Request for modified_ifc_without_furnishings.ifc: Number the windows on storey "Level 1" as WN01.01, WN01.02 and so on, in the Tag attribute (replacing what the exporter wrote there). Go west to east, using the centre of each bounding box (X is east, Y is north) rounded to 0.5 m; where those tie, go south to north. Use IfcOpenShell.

First a look at what the model holds.

```python
import ifcopenshell
import ifcopenshell.util.element
import ifcopenshell.util.placement

model = ifcopenshell.open("modified_ifc_without_furnishings.ifc")
print(model.schema)
storey = next(s for s in model.by_type("IfcBuildingStorey") if s.Name == "Level 1")
windows = [e for e in ifcopenshell.util.element.get_decomposition(storey) if e.is_a("IfcWindow")]
for e in sorted(windows, key=lambda e: e.id()):
    origin = ifcopenshell.util.placement.get_local_placement(e.ObjectPlacement)[:3, 3]
    print(e.id(), e.Tag, e.Name, origin.round(2) + 0.0, sep=" | ")
```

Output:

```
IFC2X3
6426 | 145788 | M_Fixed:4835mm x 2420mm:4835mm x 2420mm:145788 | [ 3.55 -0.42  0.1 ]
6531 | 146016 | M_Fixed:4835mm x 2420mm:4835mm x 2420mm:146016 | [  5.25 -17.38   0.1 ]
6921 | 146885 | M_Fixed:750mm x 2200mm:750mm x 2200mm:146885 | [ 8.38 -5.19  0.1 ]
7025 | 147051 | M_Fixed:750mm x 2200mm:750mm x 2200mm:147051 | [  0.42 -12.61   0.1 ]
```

```python
import ifcopenshell
import ifcopenshell.geom
import ifcopenshell.util.element
import ifcopenshell.util.shape

model = ifcopenshell.open("modified_ifc_without_furnishings.ifc")
settings = ifcopenshell.geom.settings()
settings.set("use-world-coords", True)


def centre(element):
    shape = ifcopenshell.geom.create_shape(settings, element)
    return ifcopenshell.util.shape.get_bbox_centroid(shape.geometry)


storey = next(s for s in model.by_type("IfcBuildingStorey") if s.Name == "Level 1")
windows = [e for e in ifcopenshell.util.element.get_decomposition(storey) if e.is_a("IfcWindow")]

# Insertion points can sit at a corner or the storey origin, so sort by the geometry (in metres).
centres = {e: centre(e) for e in windows}
windows.sort(key=lambda e: (round(centres[e][0] / 0.5), centres[e][1]))

for i, e in enumerate(windows, start=1):
    number = f"WN01.{i:02d}"
    e.Tag = number
    print(e.id(), number)

model.write("modified_ifc_without_furnishings-out.ifc")
```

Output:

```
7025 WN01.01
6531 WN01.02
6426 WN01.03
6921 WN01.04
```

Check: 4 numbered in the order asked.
